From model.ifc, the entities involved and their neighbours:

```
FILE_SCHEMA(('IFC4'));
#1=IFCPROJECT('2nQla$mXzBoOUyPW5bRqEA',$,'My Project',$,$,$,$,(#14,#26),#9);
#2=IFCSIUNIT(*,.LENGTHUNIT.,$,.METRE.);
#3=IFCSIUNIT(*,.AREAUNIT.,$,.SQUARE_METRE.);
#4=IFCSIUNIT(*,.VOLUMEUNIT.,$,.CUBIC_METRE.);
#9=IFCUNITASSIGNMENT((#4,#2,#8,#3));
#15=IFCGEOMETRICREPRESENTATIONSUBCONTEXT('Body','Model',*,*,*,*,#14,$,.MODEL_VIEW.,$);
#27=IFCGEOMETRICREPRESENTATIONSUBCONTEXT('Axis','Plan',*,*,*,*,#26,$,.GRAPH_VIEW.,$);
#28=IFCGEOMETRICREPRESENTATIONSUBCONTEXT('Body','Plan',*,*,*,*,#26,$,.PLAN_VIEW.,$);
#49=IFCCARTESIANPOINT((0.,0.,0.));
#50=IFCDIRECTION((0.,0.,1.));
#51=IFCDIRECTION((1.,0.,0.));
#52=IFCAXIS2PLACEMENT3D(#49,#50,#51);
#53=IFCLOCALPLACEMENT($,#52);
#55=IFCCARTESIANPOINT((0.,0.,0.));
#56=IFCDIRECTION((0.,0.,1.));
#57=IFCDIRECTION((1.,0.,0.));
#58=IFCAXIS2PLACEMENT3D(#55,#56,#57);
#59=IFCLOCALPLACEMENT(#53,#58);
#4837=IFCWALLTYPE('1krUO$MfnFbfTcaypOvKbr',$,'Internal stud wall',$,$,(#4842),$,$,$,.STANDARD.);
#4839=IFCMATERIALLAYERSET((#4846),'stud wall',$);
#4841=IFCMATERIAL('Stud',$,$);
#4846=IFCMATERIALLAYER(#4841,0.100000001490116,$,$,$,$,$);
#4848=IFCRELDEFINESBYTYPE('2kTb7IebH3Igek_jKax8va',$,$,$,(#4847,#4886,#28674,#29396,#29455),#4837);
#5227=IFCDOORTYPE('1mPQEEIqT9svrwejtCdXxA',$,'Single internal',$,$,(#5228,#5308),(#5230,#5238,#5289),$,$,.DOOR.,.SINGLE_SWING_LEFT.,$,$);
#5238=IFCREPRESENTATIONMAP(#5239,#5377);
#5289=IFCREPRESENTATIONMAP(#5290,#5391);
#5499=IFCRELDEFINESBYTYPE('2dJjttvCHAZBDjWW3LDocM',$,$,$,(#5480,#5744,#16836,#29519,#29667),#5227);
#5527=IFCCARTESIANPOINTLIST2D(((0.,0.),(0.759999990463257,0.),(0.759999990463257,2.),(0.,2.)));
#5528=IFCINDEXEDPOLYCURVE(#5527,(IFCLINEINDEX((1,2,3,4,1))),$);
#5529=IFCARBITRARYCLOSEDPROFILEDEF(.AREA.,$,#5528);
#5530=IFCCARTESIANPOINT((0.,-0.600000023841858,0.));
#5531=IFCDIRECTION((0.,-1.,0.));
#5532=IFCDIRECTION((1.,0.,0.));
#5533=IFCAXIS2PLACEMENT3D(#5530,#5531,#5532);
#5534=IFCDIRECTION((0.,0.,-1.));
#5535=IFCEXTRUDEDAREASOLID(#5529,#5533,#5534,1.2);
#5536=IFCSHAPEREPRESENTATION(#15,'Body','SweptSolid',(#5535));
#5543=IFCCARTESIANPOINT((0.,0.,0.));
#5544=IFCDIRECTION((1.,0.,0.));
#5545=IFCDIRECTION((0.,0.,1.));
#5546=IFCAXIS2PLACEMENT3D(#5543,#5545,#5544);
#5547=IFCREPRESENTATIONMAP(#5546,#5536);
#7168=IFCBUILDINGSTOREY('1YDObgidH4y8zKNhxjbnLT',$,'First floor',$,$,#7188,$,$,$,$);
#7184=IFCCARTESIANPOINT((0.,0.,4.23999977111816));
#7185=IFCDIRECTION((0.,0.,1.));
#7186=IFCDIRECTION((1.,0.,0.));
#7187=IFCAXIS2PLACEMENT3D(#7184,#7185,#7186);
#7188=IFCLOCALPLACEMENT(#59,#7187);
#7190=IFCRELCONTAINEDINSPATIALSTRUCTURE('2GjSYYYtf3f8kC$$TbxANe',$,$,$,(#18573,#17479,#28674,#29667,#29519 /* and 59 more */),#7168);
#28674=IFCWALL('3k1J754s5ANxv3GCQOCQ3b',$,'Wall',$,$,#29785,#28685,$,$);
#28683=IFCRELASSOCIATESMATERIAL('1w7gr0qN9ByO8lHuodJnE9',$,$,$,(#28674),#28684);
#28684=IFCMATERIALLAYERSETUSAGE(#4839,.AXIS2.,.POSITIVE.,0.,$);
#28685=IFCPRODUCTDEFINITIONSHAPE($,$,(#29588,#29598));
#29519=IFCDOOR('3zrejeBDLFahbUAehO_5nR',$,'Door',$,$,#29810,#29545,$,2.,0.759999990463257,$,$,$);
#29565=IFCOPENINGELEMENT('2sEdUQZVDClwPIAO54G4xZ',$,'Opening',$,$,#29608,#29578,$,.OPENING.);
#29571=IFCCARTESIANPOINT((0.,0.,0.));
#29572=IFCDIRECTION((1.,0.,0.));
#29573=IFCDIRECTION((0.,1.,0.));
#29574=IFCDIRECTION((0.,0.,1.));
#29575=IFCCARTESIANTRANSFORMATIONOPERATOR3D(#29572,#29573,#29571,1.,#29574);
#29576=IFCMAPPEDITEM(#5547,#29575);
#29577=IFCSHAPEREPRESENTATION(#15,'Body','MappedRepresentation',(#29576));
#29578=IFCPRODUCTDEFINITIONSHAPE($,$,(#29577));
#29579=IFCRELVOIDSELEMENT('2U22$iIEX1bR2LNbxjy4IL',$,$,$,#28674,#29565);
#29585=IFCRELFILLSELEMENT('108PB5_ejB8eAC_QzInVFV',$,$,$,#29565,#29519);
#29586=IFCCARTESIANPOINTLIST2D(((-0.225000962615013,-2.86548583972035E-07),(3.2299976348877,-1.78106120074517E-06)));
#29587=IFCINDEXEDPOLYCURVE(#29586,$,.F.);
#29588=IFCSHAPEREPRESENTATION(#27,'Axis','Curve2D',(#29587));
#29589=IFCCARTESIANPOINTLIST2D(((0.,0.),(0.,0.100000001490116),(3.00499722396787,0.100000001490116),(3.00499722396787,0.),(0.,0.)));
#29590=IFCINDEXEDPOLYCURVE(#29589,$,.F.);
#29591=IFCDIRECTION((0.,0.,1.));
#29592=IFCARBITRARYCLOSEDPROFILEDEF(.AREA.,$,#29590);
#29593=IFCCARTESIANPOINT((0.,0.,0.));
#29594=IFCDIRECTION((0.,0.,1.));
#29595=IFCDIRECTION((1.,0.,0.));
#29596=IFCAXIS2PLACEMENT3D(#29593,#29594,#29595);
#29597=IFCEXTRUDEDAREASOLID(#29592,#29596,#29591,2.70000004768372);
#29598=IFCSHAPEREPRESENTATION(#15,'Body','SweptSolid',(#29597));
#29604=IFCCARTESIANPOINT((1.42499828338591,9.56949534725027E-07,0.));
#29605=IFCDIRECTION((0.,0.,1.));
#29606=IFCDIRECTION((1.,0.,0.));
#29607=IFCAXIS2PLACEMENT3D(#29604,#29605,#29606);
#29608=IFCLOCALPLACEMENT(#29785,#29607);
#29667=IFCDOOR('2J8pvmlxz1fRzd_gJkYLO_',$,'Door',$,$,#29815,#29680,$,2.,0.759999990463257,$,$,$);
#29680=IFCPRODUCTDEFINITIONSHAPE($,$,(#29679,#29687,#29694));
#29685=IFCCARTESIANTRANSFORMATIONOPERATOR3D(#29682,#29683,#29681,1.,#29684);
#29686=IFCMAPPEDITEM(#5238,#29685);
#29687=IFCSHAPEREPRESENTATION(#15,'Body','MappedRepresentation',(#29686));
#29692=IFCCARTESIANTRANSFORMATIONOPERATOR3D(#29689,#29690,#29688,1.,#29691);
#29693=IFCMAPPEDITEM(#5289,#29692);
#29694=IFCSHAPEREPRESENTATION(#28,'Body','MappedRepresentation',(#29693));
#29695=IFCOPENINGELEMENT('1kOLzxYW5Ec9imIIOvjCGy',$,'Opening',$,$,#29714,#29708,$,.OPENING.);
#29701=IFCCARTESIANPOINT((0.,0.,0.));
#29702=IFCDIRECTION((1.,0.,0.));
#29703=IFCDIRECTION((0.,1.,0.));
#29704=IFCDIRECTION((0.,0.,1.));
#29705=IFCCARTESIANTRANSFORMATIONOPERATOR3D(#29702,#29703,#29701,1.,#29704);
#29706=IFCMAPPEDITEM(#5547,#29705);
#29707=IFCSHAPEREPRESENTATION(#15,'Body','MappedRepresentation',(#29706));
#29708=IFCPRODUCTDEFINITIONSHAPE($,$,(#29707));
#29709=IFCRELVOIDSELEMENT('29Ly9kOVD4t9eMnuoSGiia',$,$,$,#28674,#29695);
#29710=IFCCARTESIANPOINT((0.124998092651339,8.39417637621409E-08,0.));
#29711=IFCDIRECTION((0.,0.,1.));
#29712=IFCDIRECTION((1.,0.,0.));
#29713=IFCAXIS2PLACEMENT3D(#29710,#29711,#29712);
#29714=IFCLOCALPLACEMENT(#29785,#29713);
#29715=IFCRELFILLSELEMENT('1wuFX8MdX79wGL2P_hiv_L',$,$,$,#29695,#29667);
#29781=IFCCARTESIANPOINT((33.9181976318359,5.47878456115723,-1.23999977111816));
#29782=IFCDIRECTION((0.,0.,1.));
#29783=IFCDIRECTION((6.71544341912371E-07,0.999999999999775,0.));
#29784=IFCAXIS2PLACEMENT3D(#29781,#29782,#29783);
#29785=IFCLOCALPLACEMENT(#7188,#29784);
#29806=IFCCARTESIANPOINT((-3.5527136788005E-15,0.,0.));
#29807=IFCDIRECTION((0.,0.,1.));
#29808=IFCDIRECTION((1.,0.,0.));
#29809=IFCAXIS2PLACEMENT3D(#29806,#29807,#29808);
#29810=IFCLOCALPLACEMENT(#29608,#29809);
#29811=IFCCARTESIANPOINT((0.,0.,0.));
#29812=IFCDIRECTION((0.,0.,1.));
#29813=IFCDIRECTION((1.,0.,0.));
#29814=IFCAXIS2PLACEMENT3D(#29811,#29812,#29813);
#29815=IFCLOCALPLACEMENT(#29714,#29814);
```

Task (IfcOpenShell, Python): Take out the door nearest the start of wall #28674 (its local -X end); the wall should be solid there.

```python
import ifcopenshell
import ifcopenshell.api.feature
import ifcopenshell.api.root
import ifcopenshell.geom
import ifcopenshell.util.shape

model = ifcopenshell.open("model.ifc")
settings = ifcopenshell.geom.settings()


def volume(element):
    """Net volume in cubic metres, openings subtracted."""
    shape = ifcopenshell.geom.create_shape(settings, element)
    return ifcopenshell.util.shape.get_volume(shape.geometry)


door = model.by_guid("2J8pvmlxz1fRzd_gJkYLO_")
opening = door.FillsVoids[0].RelatingOpeningElement
wall = opening.VoidsElements[0].RelatingBuildingElement
before = volume(wall)

ifcopenshell.api.root.remove_product(model, product=door)
ifcopenshell.api.feature.remove_feature(model, feature=opening)

after = volume(wall)

print(f"wall volume {before:.3f} -> {after:.3f} m3")

model.write("model_edited.ifc")
```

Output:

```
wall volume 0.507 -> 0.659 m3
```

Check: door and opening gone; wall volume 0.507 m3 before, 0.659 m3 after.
